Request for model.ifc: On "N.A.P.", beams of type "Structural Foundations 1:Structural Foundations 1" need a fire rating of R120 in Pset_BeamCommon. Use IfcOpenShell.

First a look at what the model holds.

```python
import ifcopenshell
import ifcopenshell.util.element

model = ifcopenshell.open("model.ifc")
print(model.schema)
storey = next(s for s in model.by_type("IfcBuildingStorey") if s.Name == "N.A.P.")
beams = [e for e in ifcopenshell.util.element.get_decomposition(storey) if e.is_a("IfcBeam")]
seen = {}
for e in beams:
    element_type = ifcopenshell.util.element.get_type(e)
    key = (element_type.Name if element_type != e and element_type else None, ifcopenshell.util.element.get_pset(e, "Pset_BeamCommon", "FireRating"))
    seen[key] = seen.get(key, 0) + 1
for (name, value), count in sorted(seen.items(), key=str):
    print(count, "x", name, "|", value)
```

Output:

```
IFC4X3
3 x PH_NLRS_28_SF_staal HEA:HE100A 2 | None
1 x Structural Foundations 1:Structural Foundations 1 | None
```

```python
import ifcopenshell
import ifcopenshell.api.pset
import ifcopenshell.util.element

model = ifcopenshell.open("model.ifc")

storey = next(s for s in model.by_type("IfcBuildingStorey") if s.Name == "N.A.P.")
beams = [e for e in ifcopenshell.util.element.get_decomposition(storey) if e.is_a("IfcBeam")]

count = 0
for e in beams:
    element_type = ifcopenshell.util.element.get_type(e)
    if element_type in (None, e) or element_type.Name != "Structural Foundations 1:Structural Foundations 1":
        continue
    # add_pset returns the element's existing set when there is one.
    pset = ifcopenshell.api.pset.add_pset(model, product=e, name="Pset_BeamCommon")
    ifcopenshell.api.pset.edit_pset(model, pset=pset, properties={"FireRating": "R120"})
    count += 1

print(count, "beams updated")

model.write("model_updated.ifc")
```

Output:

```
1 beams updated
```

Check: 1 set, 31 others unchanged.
